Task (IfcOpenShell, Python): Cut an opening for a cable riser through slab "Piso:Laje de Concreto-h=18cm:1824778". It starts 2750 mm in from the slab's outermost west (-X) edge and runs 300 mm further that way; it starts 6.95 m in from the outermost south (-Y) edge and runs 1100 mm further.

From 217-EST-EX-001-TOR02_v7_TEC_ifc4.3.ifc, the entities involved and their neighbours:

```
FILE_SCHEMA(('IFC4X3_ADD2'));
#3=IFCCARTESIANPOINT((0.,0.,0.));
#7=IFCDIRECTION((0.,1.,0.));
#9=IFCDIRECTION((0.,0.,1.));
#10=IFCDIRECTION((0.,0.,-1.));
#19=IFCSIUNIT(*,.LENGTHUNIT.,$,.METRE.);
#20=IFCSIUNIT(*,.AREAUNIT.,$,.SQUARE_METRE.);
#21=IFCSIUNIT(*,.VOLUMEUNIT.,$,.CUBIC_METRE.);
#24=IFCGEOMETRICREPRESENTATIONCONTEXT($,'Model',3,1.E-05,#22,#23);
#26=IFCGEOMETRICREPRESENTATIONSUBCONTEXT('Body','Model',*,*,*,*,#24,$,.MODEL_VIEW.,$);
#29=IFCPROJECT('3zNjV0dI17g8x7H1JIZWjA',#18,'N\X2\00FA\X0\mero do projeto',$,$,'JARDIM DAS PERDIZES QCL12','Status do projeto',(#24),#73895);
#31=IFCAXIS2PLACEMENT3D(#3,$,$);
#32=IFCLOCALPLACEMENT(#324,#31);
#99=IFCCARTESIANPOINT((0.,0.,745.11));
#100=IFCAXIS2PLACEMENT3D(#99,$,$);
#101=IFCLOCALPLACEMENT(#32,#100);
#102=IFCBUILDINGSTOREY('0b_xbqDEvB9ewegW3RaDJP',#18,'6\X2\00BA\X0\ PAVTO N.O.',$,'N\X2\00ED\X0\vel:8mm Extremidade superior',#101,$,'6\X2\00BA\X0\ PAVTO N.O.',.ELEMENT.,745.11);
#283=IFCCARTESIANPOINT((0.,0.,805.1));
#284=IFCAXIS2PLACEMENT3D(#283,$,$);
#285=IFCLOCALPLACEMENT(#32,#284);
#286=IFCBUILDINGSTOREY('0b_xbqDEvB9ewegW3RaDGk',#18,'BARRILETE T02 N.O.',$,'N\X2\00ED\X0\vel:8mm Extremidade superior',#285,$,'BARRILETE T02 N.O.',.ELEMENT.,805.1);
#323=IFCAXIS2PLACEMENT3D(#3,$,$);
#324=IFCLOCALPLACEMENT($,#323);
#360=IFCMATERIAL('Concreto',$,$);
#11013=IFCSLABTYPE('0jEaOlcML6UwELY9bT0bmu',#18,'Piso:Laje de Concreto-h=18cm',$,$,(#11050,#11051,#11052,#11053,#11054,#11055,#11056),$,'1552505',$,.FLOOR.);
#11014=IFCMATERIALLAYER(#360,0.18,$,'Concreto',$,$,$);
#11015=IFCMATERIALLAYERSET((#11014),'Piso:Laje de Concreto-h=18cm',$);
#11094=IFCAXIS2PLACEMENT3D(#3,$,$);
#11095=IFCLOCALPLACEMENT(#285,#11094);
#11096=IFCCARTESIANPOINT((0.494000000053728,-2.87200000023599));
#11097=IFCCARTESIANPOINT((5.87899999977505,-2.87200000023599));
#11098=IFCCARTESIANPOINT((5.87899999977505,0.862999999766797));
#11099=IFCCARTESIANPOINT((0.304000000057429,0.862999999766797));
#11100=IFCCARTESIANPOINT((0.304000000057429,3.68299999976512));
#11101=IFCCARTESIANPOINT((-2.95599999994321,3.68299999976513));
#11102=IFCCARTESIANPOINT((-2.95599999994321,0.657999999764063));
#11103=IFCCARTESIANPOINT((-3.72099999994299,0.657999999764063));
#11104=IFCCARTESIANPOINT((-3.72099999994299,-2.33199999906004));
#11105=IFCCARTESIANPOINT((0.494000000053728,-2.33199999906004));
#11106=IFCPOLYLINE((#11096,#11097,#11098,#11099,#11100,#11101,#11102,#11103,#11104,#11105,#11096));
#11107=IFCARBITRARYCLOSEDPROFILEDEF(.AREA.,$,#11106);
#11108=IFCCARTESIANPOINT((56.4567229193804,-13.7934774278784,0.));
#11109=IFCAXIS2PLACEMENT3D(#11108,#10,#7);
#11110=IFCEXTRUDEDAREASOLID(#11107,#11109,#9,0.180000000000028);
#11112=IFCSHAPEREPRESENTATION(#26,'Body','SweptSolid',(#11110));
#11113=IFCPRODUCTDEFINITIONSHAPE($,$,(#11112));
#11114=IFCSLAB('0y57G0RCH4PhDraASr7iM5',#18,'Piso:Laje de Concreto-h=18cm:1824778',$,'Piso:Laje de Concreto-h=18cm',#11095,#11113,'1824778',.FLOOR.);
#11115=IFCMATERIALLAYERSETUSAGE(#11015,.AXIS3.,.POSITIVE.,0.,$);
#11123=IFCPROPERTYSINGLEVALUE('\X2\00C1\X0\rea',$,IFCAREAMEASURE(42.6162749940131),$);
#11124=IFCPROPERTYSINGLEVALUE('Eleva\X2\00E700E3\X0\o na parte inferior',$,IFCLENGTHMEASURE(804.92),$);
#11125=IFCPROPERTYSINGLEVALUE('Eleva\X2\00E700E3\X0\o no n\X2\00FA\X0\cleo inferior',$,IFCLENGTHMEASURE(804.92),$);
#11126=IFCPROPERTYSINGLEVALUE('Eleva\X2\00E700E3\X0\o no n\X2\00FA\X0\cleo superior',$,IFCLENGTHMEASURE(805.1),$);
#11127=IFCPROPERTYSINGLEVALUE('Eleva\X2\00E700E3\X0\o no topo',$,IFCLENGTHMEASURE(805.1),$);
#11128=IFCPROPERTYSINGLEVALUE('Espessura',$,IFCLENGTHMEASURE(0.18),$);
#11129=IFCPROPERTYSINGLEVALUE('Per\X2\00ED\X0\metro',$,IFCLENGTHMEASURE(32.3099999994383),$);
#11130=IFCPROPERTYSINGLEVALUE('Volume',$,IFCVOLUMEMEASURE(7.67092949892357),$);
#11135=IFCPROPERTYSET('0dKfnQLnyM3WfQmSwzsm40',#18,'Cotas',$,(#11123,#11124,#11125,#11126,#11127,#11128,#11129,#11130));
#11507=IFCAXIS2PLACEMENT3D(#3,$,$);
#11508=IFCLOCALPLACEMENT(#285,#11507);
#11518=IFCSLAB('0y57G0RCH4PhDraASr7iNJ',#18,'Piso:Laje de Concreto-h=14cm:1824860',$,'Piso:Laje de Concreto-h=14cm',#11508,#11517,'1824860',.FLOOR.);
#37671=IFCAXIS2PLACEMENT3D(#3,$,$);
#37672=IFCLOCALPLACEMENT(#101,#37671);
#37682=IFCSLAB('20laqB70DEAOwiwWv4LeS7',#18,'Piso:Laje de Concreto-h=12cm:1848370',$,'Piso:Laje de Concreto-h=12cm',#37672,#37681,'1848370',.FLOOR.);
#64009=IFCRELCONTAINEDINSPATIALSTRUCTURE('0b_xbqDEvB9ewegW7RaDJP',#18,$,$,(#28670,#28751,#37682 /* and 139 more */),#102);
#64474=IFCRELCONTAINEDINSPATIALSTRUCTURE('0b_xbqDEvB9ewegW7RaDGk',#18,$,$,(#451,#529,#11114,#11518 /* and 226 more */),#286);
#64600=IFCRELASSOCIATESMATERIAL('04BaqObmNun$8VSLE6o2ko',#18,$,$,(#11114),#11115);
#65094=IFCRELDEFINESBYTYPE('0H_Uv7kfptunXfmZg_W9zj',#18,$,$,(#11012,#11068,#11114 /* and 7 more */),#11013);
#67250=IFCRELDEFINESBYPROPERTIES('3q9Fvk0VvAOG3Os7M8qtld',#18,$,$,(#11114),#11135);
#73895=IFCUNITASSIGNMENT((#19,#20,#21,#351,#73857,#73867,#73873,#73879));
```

```python
import numpy as np
import ifcopenshell
import ifcopenshell.api.feature
import ifcopenshell.api.geometry
import ifcopenshell.api.pset
import ifcopenshell.api.root
import ifcopenshell.geom
import ifcopenshell.util.element
import ifcopenshell.util.placement
import ifcopenshell.util.representation
import ifcopenshell.util.shape
import ifcopenshell.util.unit

model = ifcopenshell.open("217-EST-EX-001-TOR02_v7_TEC_ifc4.3.ifc")
unit_scale = ifcopenshell.util.unit.calculate_unit_scale(model)
area_scale = ifcopenshell.util.unit.calculate_unit_scale(model, "AREAUNIT")
volume_scale = ifcopenshell.util.unit.calculate_unit_scale(model, "VOLUMEUNIT")
settings = ifcopenshell.geom.settings()


def volume(element):
    """Net volume in cubic metres, openings subtracted."""
    shape = ifcopenshell.geom.create_shape(settings, element)
    return ifcopenshell.util.shape.get_volume(shape.geometry)


slab = model.by_guid("0y57G0RCH4PhDraASr7iM5")
before = volume(slab)

# Extent in the slab's own axes, in metres. The edges named are its -X and -Y sides.
slab_shape = ifcopenshell.geom.create_shape(settings, slab)
vertices = ifcopenshell.util.shape.get_vertices(slab_shape.geometry)
x_min, y_min, bottom = vertices.min(axis=0)
top = vertices[:, 2].max()

opening = ifcopenshell.api.root.create_entity(model, ifc_class="IfcOpeningElement", name="Cable riser opening", predefined_type="OPENING")
context = ifcopenshell.util.representation.get_context(model, "Model", "Body", "MODEL_VIEW")
width, depth = 0.3, 1.1
outline = [(0.0, 0.0), (width, 0.0), (width, depth), (0.0, depth), (0.0, 0.0)]
# Overshoot both faces by 50 mm so the cut is clean.
shape = ifcopenshell.api.geometry.add_slab_representation(
    model, context=context, depth=top - bottom + 0.1, polyline=outline
)
ifcopenshell.api.geometry.assign_representation(model, product=opening, representation=shape)

matrix = ifcopenshell.util.placement.get_local_placement(slab.ObjectPlacement)
matrix[:, 3] = matrix @ np.append(np.array([x_min + 2.75, y_min + 6.95, bottom - 0.05]) / unit_scale, 1.0)
ifcopenshell.api.geometry.edit_object_placement(model, product=opening, matrix=matrix, is_si=False)
ifcopenshell.api.feature.add_feature(model, feature=opening, element=slab)

after = volume(slab)

# Update the slab's stored quantities.
pset = model.by_id(ifcopenshell.util.element.get_pset(slab, "Cotas", should_inherit=False)["id"])
ifcopenshell.api.pset.edit_pset(model, pset=pset, properties={
    "Área": model.create_entity("IfcAreaMeasure", after / (top - bottom) / area_scale),
    "Volume": model.create_entity("IfcVolumeMeasure", after / volume_scale),
})

print(f"slab volume {before:.3f} -> {after:.3f} m3")

model.write("217-EST-EX-001-TOR02_v7_TEC_ifc4.3_v2.ifc")
```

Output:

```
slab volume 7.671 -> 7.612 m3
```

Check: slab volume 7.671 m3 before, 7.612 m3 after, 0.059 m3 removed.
